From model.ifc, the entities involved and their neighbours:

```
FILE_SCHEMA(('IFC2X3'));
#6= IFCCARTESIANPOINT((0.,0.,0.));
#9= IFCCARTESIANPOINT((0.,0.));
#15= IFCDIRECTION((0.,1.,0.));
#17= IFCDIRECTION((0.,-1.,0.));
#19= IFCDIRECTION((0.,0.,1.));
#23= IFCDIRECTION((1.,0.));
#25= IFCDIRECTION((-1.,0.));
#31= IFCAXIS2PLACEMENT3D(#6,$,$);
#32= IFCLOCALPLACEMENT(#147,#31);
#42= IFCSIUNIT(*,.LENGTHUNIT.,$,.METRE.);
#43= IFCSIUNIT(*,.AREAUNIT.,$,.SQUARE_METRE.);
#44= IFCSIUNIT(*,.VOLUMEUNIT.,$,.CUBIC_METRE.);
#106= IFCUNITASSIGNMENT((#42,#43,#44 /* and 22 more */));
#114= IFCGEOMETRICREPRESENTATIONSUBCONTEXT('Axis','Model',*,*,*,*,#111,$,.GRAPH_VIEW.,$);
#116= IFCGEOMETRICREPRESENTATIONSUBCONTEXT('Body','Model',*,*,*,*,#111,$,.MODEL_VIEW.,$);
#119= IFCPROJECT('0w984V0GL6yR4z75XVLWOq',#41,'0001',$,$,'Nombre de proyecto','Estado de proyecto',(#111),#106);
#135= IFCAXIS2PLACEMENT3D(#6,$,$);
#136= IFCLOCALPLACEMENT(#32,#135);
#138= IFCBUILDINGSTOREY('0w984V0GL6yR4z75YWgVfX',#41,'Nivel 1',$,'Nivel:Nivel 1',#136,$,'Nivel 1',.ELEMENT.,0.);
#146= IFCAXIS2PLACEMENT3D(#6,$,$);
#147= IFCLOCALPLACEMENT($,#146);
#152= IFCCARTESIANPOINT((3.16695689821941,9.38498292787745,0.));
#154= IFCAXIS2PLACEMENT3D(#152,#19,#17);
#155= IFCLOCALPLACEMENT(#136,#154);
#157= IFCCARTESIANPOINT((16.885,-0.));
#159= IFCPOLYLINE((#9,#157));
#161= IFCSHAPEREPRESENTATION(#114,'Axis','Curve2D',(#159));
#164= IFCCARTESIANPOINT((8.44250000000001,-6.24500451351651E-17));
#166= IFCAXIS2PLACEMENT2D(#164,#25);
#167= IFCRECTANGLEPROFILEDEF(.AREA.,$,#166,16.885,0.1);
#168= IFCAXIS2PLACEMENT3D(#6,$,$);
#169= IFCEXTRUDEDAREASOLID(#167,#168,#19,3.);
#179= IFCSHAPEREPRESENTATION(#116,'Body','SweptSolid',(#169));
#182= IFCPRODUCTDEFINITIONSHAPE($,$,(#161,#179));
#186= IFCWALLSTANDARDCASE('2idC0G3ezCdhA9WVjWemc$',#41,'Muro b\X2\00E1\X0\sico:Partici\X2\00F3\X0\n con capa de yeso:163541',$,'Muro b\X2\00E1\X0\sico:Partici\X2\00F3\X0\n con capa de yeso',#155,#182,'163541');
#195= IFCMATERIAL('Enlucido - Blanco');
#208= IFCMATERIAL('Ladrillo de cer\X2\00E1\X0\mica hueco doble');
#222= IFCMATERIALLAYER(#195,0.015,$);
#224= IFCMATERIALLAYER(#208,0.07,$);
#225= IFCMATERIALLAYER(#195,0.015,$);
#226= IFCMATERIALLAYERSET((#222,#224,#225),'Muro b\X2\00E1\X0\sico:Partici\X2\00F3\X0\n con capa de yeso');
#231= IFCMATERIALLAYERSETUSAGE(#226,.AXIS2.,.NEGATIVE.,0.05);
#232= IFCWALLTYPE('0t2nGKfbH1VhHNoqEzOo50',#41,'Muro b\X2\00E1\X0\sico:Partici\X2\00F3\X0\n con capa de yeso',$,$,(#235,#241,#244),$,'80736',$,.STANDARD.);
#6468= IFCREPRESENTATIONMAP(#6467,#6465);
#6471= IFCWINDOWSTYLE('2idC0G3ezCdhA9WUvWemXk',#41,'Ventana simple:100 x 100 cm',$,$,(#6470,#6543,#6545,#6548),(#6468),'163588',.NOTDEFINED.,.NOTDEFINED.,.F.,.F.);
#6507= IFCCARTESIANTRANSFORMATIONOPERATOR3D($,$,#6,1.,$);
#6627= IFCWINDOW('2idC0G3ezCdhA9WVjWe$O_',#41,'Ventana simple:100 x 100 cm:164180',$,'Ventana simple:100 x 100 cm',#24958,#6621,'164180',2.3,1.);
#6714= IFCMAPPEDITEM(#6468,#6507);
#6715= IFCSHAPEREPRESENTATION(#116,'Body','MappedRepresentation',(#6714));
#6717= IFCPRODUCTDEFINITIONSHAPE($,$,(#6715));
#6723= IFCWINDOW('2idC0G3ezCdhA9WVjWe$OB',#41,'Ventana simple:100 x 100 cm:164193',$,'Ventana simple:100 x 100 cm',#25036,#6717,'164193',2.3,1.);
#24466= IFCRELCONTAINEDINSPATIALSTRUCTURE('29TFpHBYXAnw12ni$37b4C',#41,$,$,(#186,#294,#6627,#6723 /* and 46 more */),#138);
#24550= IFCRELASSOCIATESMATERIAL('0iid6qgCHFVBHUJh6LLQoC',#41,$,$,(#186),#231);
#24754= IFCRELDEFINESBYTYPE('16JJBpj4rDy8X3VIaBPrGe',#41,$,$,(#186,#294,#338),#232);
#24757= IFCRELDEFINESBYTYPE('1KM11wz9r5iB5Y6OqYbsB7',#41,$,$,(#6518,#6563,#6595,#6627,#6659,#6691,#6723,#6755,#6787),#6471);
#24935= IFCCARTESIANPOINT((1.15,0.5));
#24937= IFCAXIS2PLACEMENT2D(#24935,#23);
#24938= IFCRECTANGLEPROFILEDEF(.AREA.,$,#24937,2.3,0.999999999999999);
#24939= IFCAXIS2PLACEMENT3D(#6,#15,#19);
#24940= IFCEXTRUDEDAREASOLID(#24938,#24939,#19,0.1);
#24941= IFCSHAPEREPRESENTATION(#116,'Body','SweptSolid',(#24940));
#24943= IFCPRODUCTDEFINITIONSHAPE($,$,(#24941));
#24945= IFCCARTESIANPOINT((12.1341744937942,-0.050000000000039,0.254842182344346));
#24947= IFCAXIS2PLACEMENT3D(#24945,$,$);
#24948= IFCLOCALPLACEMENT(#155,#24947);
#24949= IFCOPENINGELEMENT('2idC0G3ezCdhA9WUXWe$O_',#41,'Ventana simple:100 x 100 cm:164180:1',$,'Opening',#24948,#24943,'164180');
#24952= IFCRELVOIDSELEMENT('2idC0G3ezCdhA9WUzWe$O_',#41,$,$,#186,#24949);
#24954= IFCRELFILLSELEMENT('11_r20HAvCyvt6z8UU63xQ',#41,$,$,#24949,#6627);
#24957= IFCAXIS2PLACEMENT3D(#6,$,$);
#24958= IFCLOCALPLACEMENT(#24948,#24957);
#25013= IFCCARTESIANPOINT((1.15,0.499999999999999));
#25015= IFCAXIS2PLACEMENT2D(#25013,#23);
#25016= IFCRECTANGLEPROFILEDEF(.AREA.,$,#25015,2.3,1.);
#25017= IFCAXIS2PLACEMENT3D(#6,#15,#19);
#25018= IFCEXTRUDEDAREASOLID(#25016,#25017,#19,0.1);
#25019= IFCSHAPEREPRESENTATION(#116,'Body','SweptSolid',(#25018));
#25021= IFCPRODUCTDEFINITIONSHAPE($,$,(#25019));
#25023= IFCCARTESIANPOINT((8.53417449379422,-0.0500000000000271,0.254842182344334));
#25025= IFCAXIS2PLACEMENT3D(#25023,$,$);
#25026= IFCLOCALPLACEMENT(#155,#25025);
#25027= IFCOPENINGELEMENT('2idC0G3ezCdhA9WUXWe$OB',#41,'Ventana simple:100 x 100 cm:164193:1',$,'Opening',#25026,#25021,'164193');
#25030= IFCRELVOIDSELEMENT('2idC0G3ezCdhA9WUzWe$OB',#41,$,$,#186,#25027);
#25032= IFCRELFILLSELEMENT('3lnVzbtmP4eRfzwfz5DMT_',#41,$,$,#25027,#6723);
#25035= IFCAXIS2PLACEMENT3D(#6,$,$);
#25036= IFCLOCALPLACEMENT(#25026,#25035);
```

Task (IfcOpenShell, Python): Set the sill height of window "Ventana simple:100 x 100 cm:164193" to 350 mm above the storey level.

```python
import numpy as np
import ifcopenshell
import ifcopenshell.api.geometry
import ifcopenshell.geom
import ifcopenshell.util.element
import ifcopenshell.util.placement
import ifcopenshell.util.shape
import ifcopenshell.util.unit

model = ifcopenshell.open("model.ifc")
unit_scale = ifcopenshell.util.unit.calculate_unit_scale(model)

window = model.by_id(6723)
opening = window.FillsVoids[0].RelatingOpeningElement
storey = ifcopenshell.util.element.get_container(window, ifc_class="IfcBuildingStorey")
level = ifcopenshell.util.placement.get_local_placement(storey.ObjectPlacement)[2, 3]

# The opening's origin need not be at the sill, so measure its lowest point.
shape = ifcopenshell.geom.create_shape(ifcopenshell.geom.settings(), opening)
bottom = ifcopenshell.util.shape.get_shape_bottom_elevation(shape, shape.geometry) / unit_scale
dz = level + 0.35 / unit_scale - bottom

shift = np.array([0.0, 0.0, dz])
# The window is placed relative to its opening, so it follows when the opening moves.
matrix = ifcopenshell.util.placement.get_local_placement(opening.ObjectPlacement)
matrix[:3, 3] += shift
ifcopenshell.api.geometry.edit_object_placement(
    model, product=opening, matrix=matrix, is_si=False, should_transform_children=True
)

print(f"moved by {dz * unit_scale:+.3f} m")

model.write("model_v2.ifc")
```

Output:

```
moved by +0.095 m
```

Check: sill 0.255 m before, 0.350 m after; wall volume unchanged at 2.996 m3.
